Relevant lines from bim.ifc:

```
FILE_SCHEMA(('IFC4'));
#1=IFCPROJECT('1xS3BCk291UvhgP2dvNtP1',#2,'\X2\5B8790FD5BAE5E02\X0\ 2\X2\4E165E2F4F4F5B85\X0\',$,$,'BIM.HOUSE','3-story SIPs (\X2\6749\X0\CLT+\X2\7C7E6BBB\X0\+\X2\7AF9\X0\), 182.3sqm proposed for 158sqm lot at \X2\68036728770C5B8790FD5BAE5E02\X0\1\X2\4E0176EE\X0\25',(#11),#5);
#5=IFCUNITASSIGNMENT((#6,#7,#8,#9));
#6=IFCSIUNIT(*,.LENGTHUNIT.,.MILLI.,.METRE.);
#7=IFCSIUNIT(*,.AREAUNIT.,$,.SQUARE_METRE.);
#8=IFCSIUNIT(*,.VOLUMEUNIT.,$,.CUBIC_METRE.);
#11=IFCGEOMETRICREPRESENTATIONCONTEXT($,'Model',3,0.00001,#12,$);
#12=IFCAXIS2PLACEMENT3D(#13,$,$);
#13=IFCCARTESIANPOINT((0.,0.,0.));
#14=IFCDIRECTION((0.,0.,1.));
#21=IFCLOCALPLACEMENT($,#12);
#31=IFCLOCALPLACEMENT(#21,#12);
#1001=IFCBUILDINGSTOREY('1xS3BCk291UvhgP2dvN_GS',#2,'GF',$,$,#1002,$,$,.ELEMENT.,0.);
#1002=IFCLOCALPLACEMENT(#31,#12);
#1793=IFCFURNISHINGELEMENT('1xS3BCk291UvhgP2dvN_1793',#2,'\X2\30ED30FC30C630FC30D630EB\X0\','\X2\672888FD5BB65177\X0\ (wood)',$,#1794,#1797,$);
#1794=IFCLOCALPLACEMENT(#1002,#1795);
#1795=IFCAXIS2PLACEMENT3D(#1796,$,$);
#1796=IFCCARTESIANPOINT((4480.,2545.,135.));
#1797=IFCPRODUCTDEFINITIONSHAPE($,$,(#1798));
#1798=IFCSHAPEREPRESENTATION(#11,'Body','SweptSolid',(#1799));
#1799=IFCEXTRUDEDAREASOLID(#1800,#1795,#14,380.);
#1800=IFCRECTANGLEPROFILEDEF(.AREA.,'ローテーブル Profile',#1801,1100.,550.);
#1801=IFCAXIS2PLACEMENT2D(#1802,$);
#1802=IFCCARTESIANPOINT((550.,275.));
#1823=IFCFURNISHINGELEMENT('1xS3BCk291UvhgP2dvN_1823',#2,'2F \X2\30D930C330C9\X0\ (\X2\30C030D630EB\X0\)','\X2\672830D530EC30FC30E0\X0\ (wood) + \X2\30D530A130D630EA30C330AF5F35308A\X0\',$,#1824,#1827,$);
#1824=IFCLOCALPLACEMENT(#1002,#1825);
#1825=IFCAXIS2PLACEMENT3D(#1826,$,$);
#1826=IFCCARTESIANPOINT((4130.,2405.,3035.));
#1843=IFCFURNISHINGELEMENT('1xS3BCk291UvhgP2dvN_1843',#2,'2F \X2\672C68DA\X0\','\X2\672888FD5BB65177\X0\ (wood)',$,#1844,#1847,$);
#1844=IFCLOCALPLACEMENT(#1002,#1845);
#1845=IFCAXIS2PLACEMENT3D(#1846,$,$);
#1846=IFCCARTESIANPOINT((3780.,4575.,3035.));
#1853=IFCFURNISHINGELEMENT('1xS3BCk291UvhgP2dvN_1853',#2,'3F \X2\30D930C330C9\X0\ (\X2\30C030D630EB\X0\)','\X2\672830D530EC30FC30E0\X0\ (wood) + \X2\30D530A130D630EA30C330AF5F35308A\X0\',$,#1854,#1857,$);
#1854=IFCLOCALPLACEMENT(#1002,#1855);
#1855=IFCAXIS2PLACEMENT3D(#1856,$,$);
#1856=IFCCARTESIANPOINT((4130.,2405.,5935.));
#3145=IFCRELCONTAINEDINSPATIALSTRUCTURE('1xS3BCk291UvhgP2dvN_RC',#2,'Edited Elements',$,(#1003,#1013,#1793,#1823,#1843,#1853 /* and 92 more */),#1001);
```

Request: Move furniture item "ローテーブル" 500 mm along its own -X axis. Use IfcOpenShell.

```python
import ifcopenshell
import ifcopenshell.api.geometry
import ifcopenshell.util.placement
import ifcopenshell.util.unit

model = ifcopenshell.open("bim.ifc")
unit_scale = ifcopenshell.util.unit.calculate_unit_scale(model)

item = model.by_guid("1xS3BCk291UvhgP2dvN_1793")
matrix = ifcopenshell.util.placement.get_local_placement(item.ObjectPlacement)
matrix[:3, 3] -= matrix[:3, 0] * 0.5 / unit_scale
ifcopenshell.api.geometry.edit_object_placement(model, product=item, matrix=matrix, is_si=False)

print(ifcopenshell.util.placement.get_local_placement(item.ObjectPlacement).round(3) + 0.0)

model.write("bim_rev.ifc")
```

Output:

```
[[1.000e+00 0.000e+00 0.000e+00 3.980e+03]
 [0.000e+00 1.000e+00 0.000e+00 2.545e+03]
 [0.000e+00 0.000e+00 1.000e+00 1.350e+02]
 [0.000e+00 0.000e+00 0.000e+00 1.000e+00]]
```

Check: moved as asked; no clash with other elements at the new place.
